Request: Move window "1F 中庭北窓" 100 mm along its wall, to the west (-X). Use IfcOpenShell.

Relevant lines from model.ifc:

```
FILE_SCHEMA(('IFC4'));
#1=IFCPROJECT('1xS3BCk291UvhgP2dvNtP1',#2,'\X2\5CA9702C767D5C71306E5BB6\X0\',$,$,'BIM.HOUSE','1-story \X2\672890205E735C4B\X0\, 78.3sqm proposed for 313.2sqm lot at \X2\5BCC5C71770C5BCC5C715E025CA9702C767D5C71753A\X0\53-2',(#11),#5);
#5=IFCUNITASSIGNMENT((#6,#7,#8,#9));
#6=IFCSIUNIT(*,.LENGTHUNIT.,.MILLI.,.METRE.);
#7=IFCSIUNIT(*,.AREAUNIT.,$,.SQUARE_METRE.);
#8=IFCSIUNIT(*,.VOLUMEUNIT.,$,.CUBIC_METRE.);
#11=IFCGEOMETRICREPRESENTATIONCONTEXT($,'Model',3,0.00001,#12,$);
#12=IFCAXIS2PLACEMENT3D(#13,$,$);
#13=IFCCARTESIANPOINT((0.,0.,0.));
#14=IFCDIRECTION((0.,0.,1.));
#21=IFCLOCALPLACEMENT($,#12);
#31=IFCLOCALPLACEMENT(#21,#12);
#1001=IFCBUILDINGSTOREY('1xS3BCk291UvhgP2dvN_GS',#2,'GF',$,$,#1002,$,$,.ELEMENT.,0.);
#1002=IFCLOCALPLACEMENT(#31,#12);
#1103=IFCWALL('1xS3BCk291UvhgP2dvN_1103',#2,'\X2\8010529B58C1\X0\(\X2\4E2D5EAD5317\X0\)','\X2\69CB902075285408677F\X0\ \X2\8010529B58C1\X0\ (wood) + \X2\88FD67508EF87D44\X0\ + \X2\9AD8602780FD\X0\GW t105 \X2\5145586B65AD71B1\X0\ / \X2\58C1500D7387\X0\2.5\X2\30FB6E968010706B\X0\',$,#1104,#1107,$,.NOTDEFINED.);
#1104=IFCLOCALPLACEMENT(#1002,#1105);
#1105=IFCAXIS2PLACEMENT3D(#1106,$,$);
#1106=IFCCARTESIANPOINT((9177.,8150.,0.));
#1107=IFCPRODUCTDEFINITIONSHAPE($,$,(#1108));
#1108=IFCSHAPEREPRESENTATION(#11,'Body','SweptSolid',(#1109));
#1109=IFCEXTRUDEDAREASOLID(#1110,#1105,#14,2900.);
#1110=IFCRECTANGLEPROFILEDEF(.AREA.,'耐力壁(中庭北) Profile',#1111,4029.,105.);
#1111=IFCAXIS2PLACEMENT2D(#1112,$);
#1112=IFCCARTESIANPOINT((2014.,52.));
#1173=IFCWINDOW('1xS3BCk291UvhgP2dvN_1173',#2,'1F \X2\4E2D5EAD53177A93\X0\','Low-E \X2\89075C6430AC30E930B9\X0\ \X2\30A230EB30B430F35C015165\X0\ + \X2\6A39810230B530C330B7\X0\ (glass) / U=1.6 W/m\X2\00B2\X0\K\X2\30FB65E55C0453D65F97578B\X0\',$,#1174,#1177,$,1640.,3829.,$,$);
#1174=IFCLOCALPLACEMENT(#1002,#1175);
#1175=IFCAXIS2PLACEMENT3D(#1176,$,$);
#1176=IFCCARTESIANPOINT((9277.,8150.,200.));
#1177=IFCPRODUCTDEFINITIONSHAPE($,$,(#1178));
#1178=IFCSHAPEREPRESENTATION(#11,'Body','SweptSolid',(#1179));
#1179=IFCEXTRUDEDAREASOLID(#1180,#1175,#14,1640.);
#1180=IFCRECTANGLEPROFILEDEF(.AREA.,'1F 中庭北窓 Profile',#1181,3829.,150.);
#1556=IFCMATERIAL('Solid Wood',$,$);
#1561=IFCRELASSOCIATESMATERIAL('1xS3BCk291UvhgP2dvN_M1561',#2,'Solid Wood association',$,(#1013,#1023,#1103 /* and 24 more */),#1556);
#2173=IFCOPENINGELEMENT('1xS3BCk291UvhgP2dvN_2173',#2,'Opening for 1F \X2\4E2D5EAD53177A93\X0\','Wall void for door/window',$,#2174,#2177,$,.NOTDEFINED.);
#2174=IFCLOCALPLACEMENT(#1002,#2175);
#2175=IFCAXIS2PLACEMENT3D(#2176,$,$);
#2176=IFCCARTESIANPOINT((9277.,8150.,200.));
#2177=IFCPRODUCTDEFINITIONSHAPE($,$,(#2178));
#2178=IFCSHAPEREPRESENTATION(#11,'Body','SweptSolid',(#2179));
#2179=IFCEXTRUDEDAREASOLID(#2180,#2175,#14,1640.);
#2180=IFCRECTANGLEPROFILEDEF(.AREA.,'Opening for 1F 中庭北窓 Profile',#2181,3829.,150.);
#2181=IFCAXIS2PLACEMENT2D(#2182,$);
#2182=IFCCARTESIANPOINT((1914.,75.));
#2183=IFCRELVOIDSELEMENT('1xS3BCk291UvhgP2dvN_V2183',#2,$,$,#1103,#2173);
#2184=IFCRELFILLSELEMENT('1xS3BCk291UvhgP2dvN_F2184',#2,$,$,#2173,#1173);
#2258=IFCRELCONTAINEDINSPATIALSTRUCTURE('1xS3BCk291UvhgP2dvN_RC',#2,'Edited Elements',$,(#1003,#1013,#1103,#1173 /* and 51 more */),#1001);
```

```python
import ifcopenshell
import ifcopenshell.api.geometry
import ifcopenshell.util.placement

model = ifcopenshell.open("model.ifc")

window = model.by_guid("1xS3BCk291UvhgP2dvN_1173")
opening = window.FillsVoids[0].RelatingOpeningElement
wall = opening.VoidsElements[0].RelatingBuildingElement

wall_matrix = ifcopenshell.util.placement.get_local_placement(wall.ObjectPlacement)
shift = wall_matrix[:3, 0] * -100.0
before = ifcopenshell.util.placement.get_local_placement(window.ObjectPlacement)[:3, 3].copy()

# The window is not placed relative to its opening, so move both.
for product in (opening, window):
    matrix = ifcopenshell.util.placement.get_local_placement(product.ObjectPlacement)
    matrix[:3, 3] += shift
    ifcopenshell.api.geometry.edit_object_placement(model, product=product, matrix=matrix, is_si=False)

after = ifcopenshell.util.placement.get_local_placement(window.ObjectPlacement)[:3, 3]
print("window moved by", (after - before).round(3) + 0.0)

model.write("model-out.ifc")
```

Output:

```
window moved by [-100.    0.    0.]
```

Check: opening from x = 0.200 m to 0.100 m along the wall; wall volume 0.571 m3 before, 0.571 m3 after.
